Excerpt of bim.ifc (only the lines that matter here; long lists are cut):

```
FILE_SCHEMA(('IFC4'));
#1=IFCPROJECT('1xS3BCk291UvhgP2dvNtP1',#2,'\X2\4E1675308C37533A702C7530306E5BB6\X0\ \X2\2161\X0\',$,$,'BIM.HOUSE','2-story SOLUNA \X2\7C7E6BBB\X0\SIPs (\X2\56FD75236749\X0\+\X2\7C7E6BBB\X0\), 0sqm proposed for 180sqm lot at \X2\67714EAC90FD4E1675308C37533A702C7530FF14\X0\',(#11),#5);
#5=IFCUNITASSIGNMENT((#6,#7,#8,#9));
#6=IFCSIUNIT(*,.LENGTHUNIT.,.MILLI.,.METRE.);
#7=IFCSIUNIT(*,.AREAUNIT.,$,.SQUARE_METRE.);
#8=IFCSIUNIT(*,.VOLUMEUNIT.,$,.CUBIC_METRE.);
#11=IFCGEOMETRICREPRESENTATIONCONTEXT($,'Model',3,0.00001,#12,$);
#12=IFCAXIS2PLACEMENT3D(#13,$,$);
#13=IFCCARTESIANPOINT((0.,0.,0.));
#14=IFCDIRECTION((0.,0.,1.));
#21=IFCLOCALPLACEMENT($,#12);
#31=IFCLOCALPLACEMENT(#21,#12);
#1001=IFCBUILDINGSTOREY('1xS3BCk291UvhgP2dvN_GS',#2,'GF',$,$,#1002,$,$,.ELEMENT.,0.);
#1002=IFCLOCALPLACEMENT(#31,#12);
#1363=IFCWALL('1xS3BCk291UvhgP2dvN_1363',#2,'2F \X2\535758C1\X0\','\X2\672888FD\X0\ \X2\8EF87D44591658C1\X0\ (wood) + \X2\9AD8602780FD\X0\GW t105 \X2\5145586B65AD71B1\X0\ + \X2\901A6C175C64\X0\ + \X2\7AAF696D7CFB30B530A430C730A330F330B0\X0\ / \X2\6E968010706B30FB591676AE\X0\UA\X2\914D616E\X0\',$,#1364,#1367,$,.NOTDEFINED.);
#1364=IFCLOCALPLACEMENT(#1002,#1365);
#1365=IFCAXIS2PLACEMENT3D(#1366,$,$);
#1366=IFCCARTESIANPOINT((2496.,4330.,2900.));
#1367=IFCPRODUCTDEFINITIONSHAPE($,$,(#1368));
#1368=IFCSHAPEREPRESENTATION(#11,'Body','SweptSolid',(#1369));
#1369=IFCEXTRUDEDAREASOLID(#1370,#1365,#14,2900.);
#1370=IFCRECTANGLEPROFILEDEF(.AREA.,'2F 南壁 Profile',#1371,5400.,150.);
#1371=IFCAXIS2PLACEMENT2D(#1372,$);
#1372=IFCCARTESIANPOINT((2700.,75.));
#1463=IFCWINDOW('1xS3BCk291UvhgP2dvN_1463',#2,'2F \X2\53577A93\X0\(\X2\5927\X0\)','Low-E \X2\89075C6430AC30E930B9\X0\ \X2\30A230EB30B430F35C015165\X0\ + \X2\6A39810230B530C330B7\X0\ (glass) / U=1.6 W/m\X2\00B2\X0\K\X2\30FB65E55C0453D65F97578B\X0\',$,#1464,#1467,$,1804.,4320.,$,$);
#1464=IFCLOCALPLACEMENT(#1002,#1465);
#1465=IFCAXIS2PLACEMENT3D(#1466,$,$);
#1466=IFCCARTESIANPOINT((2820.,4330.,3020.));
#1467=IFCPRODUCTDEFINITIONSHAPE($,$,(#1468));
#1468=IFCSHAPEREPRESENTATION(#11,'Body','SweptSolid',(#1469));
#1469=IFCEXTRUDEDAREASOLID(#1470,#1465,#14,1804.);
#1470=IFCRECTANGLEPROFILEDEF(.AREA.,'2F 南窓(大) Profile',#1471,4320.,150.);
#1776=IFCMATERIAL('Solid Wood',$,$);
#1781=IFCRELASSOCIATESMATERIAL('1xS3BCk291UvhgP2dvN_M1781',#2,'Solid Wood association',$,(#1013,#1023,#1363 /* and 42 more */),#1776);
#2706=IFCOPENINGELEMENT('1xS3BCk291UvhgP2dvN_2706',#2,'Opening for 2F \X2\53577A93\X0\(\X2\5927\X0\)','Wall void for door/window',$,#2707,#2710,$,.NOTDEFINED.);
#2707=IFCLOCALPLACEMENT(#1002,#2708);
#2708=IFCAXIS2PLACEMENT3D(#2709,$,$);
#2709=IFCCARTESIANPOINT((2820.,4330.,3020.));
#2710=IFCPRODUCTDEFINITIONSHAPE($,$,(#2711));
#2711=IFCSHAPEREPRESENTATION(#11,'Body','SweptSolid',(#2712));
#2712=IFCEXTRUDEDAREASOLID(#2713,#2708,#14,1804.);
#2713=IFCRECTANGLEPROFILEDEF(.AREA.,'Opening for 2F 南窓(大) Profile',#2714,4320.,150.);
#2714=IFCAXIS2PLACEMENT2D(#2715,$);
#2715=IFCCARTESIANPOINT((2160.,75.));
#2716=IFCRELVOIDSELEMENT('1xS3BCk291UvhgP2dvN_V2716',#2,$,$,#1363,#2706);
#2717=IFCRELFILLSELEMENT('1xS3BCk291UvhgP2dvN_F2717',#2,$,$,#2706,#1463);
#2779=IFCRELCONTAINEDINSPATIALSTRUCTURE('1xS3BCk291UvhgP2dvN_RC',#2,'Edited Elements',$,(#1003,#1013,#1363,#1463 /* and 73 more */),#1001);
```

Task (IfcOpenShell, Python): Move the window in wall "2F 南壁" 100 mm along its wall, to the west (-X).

```python
import ifcopenshell
import ifcopenshell.api.geometry
import ifcopenshell.util.placement
import ifcopenshell.util.unit

model = ifcopenshell.open("bim.ifc")
unit_scale = ifcopenshell.util.unit.calculate_unit_scale(model)

window = model.by_id(1463)
opening = window.FillsVoids[0].RelatingOpeningElement
wall = opening.VoidsElements[0].RelatingBuildingElement

wall_matrix = ifcopenshell.util.placement.get_local_placement(wall.ObjectPlacement)
shift = wall_matrix[:3, 0] * -0.1 / unit_scale
before = ifcopenshell.util.placement.get_local_placement(window.ObjectPlacement)[:3, 3].copy()

# The window is not placed relative to its opening, so move both.
for product in (opening, window):
    matrix = ifcopenshell.util.placement.get_local_placement(product.ObjectPlacement)
    matrix[:3, 3] += shift
    ifcopenshell.api.geometry.edit_object_placement(model, product=product, matrix=matrix, is_si=False)

after = ifcopenshell.util.placement.get_local_placement(window.ObjectPlacement)[:3, 3]
print("window moved by", (after - before).round(3) + 0.0)

model.write("bim-out.ifc")
```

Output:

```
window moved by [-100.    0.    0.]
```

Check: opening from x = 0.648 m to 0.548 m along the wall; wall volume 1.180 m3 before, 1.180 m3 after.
